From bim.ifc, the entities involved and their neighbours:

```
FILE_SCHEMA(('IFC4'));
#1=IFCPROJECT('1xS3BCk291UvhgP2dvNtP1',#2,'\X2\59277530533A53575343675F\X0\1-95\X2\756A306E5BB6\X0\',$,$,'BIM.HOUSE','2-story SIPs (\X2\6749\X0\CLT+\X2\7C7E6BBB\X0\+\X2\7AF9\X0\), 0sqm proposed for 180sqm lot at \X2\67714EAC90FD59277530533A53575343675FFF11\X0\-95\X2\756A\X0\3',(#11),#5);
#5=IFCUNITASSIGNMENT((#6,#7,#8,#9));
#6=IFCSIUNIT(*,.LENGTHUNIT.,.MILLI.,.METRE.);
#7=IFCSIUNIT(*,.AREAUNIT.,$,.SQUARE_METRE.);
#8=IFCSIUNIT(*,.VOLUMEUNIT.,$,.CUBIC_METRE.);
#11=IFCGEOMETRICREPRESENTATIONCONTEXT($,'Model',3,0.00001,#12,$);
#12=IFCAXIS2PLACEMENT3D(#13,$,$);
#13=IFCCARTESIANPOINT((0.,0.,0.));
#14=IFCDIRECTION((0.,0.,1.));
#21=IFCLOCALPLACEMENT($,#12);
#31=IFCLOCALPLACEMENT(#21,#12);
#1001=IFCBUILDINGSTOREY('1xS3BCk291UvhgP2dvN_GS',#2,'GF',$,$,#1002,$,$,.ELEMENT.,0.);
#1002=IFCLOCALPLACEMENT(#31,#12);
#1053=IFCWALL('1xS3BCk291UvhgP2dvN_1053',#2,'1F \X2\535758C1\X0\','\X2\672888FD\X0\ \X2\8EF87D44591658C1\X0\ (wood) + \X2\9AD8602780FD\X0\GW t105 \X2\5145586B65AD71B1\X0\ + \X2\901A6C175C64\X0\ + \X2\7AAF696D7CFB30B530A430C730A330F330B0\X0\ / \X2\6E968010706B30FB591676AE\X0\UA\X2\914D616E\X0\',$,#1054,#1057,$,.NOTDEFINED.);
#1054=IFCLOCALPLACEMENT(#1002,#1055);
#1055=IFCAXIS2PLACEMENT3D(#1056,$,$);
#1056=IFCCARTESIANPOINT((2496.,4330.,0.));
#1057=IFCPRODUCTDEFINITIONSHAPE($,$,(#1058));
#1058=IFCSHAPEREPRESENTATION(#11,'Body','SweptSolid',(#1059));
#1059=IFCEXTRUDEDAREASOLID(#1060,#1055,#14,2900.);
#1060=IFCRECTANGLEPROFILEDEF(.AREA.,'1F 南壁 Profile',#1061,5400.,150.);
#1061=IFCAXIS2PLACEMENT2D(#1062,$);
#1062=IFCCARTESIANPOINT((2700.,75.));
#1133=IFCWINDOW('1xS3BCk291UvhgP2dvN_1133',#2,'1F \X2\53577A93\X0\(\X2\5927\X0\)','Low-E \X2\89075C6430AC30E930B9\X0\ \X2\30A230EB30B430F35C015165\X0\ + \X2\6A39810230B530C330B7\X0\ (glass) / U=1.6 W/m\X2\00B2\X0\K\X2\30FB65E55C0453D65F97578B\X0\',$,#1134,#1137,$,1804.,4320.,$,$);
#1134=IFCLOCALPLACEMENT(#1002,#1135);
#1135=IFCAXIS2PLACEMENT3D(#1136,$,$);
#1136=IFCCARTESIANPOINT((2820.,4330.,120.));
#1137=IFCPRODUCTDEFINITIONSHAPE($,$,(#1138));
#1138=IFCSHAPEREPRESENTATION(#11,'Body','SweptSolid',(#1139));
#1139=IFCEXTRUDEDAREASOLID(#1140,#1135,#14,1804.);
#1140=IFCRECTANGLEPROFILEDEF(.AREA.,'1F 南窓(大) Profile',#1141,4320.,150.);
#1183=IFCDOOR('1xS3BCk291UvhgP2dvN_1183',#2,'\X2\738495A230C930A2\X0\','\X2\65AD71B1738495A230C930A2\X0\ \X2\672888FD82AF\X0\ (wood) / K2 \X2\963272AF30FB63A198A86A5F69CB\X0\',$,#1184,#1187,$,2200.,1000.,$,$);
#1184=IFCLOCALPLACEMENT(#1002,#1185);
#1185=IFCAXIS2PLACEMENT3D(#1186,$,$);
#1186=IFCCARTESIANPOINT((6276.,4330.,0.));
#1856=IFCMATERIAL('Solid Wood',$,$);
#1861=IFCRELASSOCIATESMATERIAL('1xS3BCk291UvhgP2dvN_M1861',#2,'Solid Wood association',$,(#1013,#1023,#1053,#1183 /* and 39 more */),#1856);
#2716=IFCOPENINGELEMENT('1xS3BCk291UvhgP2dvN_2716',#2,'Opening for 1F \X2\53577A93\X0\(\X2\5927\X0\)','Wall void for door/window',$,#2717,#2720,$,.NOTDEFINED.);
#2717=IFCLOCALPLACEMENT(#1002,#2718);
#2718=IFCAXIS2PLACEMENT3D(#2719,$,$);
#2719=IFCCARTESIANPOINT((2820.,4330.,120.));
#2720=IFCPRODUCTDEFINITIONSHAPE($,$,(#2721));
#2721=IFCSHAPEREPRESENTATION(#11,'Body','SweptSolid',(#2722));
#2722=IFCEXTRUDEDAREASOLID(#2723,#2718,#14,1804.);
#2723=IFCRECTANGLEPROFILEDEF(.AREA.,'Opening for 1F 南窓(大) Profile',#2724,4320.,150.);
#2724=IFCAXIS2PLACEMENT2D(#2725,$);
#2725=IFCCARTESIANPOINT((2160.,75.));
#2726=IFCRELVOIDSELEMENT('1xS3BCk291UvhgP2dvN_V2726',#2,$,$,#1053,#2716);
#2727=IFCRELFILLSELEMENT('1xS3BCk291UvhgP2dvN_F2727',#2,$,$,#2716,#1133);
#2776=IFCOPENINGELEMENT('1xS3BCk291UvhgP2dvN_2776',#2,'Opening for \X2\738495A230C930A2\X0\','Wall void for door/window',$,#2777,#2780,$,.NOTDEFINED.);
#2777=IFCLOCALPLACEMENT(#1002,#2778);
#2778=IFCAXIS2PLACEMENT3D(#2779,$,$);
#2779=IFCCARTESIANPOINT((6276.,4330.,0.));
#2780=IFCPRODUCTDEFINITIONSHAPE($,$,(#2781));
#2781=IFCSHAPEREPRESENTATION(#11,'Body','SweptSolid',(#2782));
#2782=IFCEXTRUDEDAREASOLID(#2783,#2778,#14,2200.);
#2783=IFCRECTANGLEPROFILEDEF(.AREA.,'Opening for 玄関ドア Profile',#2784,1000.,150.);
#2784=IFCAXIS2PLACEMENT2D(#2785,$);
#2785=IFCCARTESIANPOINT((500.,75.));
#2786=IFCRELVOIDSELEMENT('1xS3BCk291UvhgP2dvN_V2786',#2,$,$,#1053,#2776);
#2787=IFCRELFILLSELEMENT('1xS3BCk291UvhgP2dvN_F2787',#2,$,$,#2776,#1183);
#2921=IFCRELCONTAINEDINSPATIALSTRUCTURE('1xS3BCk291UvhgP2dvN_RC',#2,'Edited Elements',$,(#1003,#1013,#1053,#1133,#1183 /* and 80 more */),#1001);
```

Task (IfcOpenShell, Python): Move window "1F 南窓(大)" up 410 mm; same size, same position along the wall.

```python
import numpy as np
import ifcopenshell
import ifcopenshell.api.geometry
import ifcopenshell.util.placement
import ifcopenshell.util.unit

model = ifcopenshell.open("bim.ifc")
unit_scale = ifcopenshell.util.unit.calculate_unit_scale(model)

window = model.by_id(1133)
opening = window.FillsVoids[0].RelatingOpeningElement
dz = 0.41 / unit_scale

shift = np.array([0.0, 0.0, dz])
# The window is not placed relative to its opening, so move both.
for product in (opening, window):
    matrix = ifcopenshell.util.placement.get_local_placement(product.ObjectPlacement)
    matrix[:3, 3] += shift
    ifcopenshell.api.geometry.edit_object_placement(model, product=product, matrix=matrix, is_si=False)

print(f"moved by {dz * unit_scale:+.3f} m")

model.write("bim_updated.ifc")
```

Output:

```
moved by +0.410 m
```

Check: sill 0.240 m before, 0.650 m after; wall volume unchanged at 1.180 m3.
